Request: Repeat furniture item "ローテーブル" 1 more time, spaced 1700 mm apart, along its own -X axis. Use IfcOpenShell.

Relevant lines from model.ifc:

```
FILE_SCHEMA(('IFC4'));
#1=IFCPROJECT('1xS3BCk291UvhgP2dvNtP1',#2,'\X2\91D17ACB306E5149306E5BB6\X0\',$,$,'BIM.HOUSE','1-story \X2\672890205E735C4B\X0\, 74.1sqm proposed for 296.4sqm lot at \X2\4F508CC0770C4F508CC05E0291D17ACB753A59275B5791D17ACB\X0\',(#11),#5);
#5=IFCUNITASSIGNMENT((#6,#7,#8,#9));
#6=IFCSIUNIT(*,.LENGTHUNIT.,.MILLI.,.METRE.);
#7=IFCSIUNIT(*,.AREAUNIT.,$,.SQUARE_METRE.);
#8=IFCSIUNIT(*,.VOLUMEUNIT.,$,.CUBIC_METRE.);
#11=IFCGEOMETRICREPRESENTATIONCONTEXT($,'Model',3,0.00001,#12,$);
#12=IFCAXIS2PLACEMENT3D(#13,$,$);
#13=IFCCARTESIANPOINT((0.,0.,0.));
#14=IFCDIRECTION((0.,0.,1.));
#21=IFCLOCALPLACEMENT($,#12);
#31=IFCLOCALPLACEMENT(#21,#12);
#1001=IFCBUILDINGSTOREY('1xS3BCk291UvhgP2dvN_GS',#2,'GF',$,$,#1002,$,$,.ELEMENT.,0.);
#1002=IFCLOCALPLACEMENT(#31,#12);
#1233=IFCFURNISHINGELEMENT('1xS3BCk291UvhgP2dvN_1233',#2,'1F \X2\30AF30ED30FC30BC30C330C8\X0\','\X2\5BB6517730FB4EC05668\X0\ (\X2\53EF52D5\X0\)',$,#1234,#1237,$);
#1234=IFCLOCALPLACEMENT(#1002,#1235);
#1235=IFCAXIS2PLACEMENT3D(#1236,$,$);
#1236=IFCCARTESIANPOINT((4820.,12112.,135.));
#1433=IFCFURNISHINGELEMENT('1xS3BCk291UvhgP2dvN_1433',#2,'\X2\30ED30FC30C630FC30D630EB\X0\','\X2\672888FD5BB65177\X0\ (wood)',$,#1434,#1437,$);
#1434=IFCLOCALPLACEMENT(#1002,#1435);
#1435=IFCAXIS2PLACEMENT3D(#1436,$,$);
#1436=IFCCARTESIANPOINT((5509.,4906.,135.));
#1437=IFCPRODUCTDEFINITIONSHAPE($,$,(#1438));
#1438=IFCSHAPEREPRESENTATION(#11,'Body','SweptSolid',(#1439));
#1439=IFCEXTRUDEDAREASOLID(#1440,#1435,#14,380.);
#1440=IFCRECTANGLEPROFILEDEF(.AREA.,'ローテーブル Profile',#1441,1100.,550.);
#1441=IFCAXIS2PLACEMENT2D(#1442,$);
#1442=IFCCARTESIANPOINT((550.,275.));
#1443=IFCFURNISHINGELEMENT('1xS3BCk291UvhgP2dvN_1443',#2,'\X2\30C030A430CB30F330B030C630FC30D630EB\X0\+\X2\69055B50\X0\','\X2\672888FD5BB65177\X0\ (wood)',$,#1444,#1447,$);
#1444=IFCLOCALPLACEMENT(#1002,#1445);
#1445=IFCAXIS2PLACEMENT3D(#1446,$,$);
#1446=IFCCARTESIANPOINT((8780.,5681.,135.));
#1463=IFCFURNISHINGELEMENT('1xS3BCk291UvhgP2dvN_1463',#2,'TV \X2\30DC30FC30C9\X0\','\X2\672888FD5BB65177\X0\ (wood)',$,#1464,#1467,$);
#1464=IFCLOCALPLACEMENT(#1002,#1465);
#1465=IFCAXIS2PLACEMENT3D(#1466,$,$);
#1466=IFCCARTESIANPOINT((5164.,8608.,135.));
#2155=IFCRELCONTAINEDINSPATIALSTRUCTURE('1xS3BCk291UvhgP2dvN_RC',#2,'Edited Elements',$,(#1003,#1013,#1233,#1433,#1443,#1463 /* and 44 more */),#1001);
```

```python
import ifcopenshell
import ifcopenshell.api.geometry
import ifcopenshell.api.root
import ifcopenshell.util.element
import ifcopenshell.util.placement
import ifcopenshell.util.unit

model = ifcopenshell.open("model.ifc")
unit_scale = ifcopenshell.util.unit.calculate_unit_scale(model)


def reuse_history(source, copy):
    """copy_class also copies each property set's owner history, people and application; keep the originals."""
    for rel in copy.IsDefinedBy:
        if rel.is_a("IfcRelDefinesByProperties") and (history := rel.RelatingPropertyDefinition.OwnerHistory):
            rel.RelatingPropertyDefinition.OwnerHistory = source.OwnerHistory
            ifcopenshell.util.element.remove_deep2(model, history)


source = model.by_guid("1xS3BCk291UvhgP2dvN_1433")
base = ifcopenshell.util.placement.get_local_placement(source.ObjectPlacement)
step = -base[:3, 0] * 1.7 / unit_scale

for i in range(1, 2):
    copy = ifcopenshell.api.root.copy_class(model, product=source)
    copy.Representation = ifcopenshell.util.element.copy_deep(
        model, source.Representation, exclude=["IfcGeometricRepresentationContext", "IfcRepresentationMap"]
    )
    reuse_history(source, copy)
    matrix = base.copy()
    matrix[:3, 3] += i * step
    print("added at", matrix[:3, 3].round(3) + 0.0)
    ifcopenshell.api.geometry.edit_object_placement(model, product=copy, matrix=matrix, is_si=False)

model.write("model-out.ifc")
```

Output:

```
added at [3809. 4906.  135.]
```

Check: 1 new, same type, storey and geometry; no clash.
